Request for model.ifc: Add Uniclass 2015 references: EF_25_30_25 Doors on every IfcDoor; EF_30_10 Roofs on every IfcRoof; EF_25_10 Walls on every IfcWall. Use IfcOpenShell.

First a look at what the model holds.

```python
import ifcopenshell

model = ifcopenshell.open("model.ifc")
print(model.schema)
print("classifications:", [c.Name for c in model.by_type("IfcClassification")])
for ifc_class in ("IfcDoor", "IfcRoof", "IfcStair", "IfcWall", "IfcWindow"):
    print(ifc_class, len(model.by_type(ifc_class)))
```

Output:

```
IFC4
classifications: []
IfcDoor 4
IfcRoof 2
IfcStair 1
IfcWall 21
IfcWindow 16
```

```python
import ifcopenshell
import ifcopenshell.api.classification

model = ifcopenshell.open("model.ifc")

system = ifcopenshell.api.classification.add_classification(model, classification="Uniclass 2015")

codes = {
    "IfcDoor": ("EF_25_30_25", "Doors"),
    "IfcRoof": ("EF_30_10", "Roofs"),
    "IfcWall": ("EF_25_10", "Walls"),
}
for ifc_class, (code, name) in codes.items():
    products = model.by_type(ifc_class)
    ifcopenshell.api.classification.add_reference(
        model, products=products, classification=system, identification=code, name=name
    )
    print(code, len(products))

model.write("model_rev.ifc")
```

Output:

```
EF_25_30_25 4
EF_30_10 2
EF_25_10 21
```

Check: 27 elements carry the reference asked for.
